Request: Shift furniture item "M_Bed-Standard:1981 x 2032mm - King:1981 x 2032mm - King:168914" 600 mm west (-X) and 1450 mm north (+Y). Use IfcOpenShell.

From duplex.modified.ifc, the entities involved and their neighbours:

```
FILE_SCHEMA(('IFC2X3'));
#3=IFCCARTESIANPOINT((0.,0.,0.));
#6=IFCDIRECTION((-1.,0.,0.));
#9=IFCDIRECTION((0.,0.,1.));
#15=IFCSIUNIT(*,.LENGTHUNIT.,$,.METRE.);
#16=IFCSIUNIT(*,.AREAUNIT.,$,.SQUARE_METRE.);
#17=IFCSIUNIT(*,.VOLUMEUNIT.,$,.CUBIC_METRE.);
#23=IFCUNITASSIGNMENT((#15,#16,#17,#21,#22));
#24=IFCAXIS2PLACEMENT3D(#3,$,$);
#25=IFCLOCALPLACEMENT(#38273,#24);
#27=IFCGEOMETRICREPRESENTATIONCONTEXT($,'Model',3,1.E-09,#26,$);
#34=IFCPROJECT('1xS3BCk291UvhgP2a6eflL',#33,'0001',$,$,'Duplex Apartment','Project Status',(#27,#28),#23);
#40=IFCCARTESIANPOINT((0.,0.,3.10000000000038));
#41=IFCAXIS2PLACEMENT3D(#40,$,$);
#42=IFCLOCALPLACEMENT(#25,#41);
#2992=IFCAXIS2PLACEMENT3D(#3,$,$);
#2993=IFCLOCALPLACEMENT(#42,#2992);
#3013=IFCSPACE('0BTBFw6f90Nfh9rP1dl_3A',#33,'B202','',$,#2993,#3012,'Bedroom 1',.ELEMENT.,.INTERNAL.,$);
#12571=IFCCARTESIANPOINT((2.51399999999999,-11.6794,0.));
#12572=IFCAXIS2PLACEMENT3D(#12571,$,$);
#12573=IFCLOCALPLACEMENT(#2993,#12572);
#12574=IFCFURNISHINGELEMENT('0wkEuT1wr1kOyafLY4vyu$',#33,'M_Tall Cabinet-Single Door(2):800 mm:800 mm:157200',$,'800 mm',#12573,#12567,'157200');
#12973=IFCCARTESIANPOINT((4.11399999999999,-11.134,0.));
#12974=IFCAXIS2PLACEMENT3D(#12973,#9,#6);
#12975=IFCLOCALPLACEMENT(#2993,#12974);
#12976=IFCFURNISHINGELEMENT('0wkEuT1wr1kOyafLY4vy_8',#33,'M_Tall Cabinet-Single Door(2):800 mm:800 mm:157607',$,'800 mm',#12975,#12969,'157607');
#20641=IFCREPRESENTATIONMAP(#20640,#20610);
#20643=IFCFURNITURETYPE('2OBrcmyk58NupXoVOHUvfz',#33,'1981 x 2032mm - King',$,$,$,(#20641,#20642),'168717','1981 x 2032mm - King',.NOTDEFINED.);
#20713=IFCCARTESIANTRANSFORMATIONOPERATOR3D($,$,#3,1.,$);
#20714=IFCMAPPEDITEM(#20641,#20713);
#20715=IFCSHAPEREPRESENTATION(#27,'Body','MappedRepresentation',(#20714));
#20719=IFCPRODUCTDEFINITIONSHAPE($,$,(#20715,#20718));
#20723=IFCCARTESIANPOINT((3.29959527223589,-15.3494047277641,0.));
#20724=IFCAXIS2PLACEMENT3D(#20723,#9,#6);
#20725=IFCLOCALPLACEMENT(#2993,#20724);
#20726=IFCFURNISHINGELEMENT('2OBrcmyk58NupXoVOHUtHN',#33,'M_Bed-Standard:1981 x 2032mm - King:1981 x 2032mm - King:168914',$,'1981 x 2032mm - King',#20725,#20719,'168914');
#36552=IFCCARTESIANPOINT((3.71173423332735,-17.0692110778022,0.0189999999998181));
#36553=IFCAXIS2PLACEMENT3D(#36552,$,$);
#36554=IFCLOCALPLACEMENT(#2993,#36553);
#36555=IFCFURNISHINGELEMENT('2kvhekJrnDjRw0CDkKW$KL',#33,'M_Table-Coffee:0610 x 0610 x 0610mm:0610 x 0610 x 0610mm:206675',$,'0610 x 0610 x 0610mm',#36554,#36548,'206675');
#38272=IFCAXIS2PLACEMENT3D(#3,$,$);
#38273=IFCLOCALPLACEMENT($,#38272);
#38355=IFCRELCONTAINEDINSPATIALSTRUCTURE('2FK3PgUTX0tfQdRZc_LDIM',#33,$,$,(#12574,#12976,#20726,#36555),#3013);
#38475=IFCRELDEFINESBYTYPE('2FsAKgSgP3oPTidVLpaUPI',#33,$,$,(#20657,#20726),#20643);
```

```python
import ifcopenshell
import ifcopenshell.api.geometry
import ifcopenshell.util.placement
import ifcopenshell.util.unit

model = ifcopenshell.open("duplex.modified.ifc")
unit_scale = ifcopenshell.util.unit.calculate_unit_scale(model)

item = model.by_guid("2OBrcmyk58NupXoVOHUtHN")
matrix = ifcopenshell.util.placement.get_local_placement(item.ObjectPlacement)
matrix[0, 3] -= 0.6 / unit_scale
matrix[1, 3] += 1.45 / unit_scale
ifcopenshell.api.geometry.edit_object_placement(model, product=item, matrix=matrix, is_si=False)

print(ifcopenshell.util.placement.get_local_placement(item.ObjectPlacement).round(3) + 0.0)

model.write("duplex.modified_edited.ifc")
```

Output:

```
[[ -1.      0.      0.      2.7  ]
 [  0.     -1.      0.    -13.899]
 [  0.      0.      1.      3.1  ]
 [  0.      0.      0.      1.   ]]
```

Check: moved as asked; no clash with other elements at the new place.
